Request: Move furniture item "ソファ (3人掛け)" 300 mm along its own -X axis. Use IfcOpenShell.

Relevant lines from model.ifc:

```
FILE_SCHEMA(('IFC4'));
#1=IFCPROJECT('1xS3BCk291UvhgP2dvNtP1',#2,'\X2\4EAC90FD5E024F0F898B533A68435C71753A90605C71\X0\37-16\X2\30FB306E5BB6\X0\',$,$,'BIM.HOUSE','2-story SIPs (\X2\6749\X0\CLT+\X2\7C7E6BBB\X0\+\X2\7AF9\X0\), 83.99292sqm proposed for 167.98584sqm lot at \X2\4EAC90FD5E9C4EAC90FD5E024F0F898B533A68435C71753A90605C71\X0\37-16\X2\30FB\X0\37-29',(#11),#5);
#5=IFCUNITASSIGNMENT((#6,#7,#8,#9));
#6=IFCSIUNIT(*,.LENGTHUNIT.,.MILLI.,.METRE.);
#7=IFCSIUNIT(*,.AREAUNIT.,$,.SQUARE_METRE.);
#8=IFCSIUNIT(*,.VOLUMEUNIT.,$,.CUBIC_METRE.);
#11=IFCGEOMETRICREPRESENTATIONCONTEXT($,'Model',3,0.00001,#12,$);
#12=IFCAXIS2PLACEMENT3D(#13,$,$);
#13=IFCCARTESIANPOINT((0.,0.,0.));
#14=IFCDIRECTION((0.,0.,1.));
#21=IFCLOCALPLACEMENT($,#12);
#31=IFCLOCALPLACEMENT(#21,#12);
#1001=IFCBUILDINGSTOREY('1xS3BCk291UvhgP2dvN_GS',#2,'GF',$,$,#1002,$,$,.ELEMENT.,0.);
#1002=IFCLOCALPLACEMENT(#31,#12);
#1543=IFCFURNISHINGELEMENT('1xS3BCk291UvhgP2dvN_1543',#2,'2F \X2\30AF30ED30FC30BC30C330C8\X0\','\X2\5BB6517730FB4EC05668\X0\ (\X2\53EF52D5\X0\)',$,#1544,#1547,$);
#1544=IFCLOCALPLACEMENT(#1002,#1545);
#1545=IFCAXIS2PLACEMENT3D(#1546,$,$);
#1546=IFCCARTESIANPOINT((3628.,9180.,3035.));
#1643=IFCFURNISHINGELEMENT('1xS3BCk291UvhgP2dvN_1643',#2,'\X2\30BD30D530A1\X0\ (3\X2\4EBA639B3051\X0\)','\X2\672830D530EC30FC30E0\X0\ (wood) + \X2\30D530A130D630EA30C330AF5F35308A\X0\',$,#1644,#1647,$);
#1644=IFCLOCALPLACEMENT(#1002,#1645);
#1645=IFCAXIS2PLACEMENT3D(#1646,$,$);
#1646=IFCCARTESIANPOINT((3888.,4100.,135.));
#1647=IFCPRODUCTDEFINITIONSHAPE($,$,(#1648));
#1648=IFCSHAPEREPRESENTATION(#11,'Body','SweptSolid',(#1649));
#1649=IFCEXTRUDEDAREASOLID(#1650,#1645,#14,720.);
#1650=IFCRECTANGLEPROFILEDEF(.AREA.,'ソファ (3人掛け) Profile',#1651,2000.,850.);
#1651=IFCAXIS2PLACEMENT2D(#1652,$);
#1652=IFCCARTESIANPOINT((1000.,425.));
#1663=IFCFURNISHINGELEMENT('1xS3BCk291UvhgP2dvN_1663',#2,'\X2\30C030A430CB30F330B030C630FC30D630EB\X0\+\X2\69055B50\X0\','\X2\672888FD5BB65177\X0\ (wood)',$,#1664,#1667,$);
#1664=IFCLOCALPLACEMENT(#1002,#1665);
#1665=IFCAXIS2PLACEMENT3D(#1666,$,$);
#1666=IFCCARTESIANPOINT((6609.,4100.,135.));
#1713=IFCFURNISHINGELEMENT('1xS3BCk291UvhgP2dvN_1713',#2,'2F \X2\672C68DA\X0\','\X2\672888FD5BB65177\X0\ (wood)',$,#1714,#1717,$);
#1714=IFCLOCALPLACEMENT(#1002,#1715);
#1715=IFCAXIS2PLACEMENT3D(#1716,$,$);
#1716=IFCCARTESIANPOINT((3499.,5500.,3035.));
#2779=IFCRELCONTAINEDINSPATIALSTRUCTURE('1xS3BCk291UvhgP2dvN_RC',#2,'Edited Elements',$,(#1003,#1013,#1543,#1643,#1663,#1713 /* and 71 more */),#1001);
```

```python
import ifcopenshell
import ifcopenshell.api.geometry
import ifcopenshell.util.placement
import ifcopenshell.util.unit

model = ifcopenshell.open("model.ifc")
unit_scale = ifcopenshell.util.unit.calculate_unit_scale(model)

item = model.by_guid("1xS3BCk291UvhgP2dvN_1643")
matrix = ifcopenshell.util.placement.get_local_placement(item.ObjectPlacement)
matrix[:3, 3] -= matrix[:3, 0] * 0.3 / unit_scale
ifcopenshell.api.geometry.edit_object_placement(model, product=item, matrix=matrix, is_si=False)

print(ifcopenshell.util.placement.get_local_placement(item.ObjectPlacement).round(3) + 0.0)

model.write("model_edited.ifc")
```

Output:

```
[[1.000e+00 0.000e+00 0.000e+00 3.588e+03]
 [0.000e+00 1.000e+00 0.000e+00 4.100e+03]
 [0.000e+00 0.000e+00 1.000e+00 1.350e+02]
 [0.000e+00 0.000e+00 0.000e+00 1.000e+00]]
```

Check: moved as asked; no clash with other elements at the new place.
